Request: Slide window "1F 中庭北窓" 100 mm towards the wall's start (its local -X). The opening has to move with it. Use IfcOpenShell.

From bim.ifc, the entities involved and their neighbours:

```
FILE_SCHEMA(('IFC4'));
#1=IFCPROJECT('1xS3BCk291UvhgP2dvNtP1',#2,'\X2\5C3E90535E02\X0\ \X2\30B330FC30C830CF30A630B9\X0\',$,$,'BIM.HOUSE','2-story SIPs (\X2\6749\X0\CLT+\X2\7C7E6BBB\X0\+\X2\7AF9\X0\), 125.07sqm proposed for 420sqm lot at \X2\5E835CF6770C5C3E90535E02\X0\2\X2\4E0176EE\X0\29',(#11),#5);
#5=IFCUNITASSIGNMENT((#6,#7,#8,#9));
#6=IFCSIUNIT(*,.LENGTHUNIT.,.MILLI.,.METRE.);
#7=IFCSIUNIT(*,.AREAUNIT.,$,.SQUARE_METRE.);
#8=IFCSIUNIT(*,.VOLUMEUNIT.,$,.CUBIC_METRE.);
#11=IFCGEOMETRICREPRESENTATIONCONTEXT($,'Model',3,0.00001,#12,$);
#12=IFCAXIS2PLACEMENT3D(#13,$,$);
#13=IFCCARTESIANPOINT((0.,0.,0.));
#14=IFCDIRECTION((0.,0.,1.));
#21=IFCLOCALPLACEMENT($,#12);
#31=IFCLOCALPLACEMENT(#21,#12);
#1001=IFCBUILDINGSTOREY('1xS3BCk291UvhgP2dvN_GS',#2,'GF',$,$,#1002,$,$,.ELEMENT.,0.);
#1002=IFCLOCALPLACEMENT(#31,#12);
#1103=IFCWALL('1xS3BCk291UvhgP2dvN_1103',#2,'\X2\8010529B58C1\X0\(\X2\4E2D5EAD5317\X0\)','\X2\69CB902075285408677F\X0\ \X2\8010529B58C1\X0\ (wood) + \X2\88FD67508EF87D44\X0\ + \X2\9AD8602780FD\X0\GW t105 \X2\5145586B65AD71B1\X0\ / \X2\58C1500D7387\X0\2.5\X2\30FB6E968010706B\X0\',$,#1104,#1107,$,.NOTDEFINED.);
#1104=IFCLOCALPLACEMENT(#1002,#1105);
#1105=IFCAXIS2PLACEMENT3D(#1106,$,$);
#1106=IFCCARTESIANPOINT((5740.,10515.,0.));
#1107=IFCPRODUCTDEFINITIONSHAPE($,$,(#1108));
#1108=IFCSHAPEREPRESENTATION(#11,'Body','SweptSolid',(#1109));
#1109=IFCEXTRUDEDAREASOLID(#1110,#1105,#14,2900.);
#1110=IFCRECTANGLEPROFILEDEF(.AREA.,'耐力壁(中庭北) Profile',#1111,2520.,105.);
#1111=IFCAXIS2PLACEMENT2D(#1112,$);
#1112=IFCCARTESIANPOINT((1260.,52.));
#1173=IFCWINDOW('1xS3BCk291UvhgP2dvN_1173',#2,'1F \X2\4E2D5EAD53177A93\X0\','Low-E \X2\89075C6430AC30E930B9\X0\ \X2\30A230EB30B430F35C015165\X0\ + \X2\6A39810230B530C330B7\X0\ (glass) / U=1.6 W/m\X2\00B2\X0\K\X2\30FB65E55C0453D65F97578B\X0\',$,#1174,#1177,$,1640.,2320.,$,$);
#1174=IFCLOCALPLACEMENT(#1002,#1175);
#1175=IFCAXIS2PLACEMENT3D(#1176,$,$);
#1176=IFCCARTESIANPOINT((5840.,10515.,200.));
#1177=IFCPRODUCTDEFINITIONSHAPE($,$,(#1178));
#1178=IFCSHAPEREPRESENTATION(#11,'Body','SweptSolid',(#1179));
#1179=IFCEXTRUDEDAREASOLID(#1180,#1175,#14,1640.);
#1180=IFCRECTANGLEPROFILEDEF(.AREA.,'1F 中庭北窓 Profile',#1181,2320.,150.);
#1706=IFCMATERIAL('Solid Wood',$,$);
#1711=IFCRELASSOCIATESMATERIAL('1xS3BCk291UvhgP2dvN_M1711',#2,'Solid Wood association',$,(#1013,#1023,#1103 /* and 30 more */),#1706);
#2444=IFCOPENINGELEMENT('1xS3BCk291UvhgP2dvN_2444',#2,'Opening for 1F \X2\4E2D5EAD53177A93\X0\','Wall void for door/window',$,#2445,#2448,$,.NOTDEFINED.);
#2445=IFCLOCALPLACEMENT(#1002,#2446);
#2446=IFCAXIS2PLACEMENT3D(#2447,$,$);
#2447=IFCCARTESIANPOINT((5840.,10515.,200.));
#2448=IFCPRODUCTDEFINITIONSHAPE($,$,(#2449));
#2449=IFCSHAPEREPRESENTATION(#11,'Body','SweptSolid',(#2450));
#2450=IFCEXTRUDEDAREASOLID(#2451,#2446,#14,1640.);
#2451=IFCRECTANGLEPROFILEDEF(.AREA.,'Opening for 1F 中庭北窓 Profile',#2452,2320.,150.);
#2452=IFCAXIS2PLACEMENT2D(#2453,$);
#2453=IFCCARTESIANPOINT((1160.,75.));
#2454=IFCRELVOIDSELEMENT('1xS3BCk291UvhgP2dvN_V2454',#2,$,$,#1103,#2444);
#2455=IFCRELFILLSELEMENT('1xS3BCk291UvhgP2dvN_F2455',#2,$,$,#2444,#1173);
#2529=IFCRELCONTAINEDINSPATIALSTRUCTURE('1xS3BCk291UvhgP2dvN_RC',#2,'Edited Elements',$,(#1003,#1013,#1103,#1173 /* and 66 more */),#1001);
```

```python
import ifcopenshell
import ifcopenshell.api.geometry
import ifcopenshell.util.placement
import ifcopenshell.util.unit

model = ifcopenshell.open("bim.ifc")
unit_scale = ifcopenshell.util.unit.calculate_unit_scale(model)

window = model.by_guid("1xS3BCk291UvhgP2dvN_1173")
opening = window.FillsVoids[0].RelatingOpeningElement
wall = opening.VoidsElements[0].RelatingBuildingElement

wall_matrix = ifcopenshell.util.placement.get_local_placement(wall.ObjectPlacement)
shift = wall_matrix[:3, 0] * -0.1 / unit_scale
before = ifcopenshell.util.placement.get_local_placement(window.ObjectPlacement)[:3, 3].copy()

# The window is not placed relative to its opening, so move both.
for product in (opening, window):
    matrix = ifcopenshell.util.placement.get_local_placement(product.ObjectPlacement)
    matrix[:3, 3] += shift
    ifcopenshell.api.geometry.edit_object_placement(model, product=product, matrix=matrix, is_si=False)

after = ifcopenshell.util.placement.get_local_placement(window.ObjectPlacement)[:3, 3]
print("window moved by", (after - before).round(3) + 0.0)

model.write("bim_updated.ifc")
```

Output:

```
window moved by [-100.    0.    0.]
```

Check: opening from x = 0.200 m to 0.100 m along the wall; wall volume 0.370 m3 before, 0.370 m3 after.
